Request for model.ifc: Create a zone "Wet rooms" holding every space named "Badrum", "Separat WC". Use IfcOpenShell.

First a look at what the model holds.

```python
import ifcopenshell

model = ifcopenshell.open("model.ifc")
print(model.schema)
seen = {}
for space in model.by_type("IfcSpace"):
    seen[space.LongName] = seen.get(space.LongName, 0) + 1
for name, count in sorted(seen.items(), key=str):
    print(count, "x", name)
print("zones:", [z.Name for z in model.by_type("IfcZone")][:20])
```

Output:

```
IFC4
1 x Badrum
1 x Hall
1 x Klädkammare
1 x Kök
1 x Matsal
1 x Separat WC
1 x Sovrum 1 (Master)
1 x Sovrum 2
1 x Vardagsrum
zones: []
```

```python
import ifcopenshell
import ifcopenshell.api.group
import ifcopenshell.api.root

model = ifcopenshell.open("model.ifc")

names = {"Badrum", "Separat WC"}
spaces = [s for s in model.by_type("IfcSpace") if s.LongName in names]

zone = ifcopenshell.api.root.create_entity(model, ifc_class="IfcZone", name="Wet rooms")
ifcopenshell.api.group.assign_group(model, products=spaces, group=zone)
print(len(spaces), "spaces in", zone.Name)

model.write("model-out.ifc")
```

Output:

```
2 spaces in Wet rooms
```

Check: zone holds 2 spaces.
